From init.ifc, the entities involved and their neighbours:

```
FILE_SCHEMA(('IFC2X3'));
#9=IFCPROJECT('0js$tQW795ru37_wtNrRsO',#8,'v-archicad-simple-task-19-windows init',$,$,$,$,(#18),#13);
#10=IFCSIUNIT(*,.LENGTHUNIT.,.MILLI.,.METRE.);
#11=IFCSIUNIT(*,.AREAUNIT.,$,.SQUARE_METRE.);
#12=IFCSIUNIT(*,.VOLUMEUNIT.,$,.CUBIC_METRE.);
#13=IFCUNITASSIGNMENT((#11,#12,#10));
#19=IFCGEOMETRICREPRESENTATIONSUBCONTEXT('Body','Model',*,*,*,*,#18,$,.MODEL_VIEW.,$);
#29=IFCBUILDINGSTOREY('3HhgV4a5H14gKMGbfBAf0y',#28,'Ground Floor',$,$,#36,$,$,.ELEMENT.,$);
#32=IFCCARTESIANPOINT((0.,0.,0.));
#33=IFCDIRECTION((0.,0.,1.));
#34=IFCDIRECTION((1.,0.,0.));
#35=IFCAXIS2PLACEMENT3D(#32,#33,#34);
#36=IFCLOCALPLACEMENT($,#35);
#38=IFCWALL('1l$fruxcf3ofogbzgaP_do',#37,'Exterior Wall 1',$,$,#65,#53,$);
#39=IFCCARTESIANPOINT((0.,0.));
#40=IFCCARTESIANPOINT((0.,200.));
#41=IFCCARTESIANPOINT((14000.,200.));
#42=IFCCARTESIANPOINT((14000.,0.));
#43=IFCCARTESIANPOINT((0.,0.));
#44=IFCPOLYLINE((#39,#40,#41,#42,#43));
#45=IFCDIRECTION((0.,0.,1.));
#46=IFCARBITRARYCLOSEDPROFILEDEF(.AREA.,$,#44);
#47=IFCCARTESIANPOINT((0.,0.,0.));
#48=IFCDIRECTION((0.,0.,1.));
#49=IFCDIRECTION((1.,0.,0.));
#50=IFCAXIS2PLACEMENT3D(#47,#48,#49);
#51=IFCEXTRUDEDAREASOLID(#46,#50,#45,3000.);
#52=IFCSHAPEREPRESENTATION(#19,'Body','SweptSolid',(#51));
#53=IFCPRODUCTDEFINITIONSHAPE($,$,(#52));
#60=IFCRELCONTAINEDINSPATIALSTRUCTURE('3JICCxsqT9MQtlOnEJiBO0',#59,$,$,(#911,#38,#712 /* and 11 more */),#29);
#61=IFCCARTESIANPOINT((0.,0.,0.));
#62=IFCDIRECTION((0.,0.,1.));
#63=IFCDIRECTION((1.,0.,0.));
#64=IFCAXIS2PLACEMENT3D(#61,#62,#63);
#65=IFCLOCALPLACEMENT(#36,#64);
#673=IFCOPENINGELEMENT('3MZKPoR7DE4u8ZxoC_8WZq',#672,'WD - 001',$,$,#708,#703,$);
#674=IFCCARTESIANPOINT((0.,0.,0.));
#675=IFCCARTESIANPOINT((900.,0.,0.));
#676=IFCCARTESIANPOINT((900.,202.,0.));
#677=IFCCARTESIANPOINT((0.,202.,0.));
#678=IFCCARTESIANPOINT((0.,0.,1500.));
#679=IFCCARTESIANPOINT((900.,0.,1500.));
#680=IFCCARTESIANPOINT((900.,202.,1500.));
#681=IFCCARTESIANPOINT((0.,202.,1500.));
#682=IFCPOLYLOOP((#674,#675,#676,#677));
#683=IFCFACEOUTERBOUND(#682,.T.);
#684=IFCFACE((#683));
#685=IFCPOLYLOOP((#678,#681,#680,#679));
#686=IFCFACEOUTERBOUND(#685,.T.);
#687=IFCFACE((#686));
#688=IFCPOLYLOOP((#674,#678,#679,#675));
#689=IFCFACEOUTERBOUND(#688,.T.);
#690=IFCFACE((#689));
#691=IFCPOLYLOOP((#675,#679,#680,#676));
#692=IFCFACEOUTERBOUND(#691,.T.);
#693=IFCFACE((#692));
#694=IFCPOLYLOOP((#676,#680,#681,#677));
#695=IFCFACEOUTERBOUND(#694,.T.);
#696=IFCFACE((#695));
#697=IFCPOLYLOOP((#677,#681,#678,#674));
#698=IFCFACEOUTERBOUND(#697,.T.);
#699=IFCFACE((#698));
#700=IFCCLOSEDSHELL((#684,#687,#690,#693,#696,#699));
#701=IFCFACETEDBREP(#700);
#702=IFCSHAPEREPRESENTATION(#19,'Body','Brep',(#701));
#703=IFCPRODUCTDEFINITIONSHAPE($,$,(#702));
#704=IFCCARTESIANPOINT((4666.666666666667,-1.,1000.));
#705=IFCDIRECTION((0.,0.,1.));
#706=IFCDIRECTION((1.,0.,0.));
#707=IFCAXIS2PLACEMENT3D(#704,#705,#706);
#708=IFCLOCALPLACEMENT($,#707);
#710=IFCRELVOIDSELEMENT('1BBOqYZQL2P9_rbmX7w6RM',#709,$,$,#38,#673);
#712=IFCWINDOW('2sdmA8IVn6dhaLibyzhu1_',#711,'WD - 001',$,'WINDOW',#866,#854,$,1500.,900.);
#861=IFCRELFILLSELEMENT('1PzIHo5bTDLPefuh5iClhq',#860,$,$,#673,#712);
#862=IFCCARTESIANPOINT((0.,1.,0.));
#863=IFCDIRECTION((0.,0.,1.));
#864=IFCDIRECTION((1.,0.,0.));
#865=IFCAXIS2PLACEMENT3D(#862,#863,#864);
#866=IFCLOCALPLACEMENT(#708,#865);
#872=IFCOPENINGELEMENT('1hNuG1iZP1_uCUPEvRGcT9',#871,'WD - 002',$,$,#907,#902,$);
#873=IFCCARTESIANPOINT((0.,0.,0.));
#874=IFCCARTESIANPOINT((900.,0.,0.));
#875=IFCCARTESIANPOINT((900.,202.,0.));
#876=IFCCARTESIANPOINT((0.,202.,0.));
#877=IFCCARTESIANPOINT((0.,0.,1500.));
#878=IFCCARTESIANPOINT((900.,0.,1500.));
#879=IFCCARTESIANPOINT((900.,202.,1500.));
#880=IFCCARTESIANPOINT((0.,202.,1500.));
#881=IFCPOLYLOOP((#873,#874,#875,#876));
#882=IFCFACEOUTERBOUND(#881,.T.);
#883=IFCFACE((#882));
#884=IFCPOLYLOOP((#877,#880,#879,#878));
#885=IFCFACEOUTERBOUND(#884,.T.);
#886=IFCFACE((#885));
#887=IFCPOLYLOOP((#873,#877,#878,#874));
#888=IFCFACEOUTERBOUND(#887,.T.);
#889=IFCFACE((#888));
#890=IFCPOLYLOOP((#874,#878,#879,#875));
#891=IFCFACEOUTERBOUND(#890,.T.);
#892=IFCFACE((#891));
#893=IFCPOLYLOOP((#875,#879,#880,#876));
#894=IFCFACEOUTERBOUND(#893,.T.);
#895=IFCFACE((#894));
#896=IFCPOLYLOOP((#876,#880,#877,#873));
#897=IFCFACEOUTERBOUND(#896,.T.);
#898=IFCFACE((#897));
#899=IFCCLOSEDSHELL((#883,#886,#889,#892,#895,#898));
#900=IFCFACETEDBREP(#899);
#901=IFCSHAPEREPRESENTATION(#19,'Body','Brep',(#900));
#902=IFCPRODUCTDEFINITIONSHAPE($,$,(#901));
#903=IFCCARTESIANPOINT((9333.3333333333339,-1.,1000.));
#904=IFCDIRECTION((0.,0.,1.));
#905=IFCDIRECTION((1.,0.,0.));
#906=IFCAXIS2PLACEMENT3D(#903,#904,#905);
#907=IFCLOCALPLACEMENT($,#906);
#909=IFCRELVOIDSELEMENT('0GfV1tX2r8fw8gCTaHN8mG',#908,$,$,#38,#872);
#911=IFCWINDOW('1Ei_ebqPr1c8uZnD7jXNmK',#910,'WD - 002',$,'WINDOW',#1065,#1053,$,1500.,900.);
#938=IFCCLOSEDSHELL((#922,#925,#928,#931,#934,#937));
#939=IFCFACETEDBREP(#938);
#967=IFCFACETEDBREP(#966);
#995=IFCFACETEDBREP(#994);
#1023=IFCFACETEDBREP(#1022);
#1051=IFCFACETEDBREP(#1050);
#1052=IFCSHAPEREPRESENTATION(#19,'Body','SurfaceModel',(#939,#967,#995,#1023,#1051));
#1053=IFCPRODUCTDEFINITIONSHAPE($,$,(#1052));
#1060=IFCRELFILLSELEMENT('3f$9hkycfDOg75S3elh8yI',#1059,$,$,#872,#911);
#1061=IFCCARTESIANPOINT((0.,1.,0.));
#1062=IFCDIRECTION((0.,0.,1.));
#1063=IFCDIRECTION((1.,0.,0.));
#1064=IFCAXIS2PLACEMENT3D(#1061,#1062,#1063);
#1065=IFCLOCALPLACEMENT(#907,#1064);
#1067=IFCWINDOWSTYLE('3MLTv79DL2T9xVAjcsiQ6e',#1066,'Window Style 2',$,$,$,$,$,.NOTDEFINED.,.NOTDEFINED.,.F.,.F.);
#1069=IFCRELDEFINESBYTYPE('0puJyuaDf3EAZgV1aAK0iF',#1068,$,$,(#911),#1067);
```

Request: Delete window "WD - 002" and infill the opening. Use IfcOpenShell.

```python
import ifcopenshell
import ifcopenshell.api.feature
import ifcopenshell.api.root
import ifcopenshell.geom
import ifcopenshell.util.shape

model = ifcopenshell.open("init.ifc")
settings = ifcopenshell.geom.settings()


def volume(element):
    """Net volume in cubic metres, openings subtracted."""
    shape = ifcopenshell.geom.create_shape(settings, element)
    return ifcopenshell.util.shape.get_volume(shape.geometry)


window = model.by_guid("1Ei_ebqPr1c8uZnD7jXNmK")
opening = window.FillsVoids[0].RelatingOpeningElement
wall = opening.VoidsElements[0].RelatingBuildingElement
before = volume(wall)

ifcopenshell.api.root.remove_product(model, product=window)
ifcopenshell.api.feature.remove_feature(model, feature=opening)

after = volume(wall)

print(f"wall volume {before:.3f} -> {after:.3f} m3")

model.write("init_v2.ifc")
```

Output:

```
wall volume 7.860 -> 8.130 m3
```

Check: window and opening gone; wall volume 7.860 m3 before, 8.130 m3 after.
